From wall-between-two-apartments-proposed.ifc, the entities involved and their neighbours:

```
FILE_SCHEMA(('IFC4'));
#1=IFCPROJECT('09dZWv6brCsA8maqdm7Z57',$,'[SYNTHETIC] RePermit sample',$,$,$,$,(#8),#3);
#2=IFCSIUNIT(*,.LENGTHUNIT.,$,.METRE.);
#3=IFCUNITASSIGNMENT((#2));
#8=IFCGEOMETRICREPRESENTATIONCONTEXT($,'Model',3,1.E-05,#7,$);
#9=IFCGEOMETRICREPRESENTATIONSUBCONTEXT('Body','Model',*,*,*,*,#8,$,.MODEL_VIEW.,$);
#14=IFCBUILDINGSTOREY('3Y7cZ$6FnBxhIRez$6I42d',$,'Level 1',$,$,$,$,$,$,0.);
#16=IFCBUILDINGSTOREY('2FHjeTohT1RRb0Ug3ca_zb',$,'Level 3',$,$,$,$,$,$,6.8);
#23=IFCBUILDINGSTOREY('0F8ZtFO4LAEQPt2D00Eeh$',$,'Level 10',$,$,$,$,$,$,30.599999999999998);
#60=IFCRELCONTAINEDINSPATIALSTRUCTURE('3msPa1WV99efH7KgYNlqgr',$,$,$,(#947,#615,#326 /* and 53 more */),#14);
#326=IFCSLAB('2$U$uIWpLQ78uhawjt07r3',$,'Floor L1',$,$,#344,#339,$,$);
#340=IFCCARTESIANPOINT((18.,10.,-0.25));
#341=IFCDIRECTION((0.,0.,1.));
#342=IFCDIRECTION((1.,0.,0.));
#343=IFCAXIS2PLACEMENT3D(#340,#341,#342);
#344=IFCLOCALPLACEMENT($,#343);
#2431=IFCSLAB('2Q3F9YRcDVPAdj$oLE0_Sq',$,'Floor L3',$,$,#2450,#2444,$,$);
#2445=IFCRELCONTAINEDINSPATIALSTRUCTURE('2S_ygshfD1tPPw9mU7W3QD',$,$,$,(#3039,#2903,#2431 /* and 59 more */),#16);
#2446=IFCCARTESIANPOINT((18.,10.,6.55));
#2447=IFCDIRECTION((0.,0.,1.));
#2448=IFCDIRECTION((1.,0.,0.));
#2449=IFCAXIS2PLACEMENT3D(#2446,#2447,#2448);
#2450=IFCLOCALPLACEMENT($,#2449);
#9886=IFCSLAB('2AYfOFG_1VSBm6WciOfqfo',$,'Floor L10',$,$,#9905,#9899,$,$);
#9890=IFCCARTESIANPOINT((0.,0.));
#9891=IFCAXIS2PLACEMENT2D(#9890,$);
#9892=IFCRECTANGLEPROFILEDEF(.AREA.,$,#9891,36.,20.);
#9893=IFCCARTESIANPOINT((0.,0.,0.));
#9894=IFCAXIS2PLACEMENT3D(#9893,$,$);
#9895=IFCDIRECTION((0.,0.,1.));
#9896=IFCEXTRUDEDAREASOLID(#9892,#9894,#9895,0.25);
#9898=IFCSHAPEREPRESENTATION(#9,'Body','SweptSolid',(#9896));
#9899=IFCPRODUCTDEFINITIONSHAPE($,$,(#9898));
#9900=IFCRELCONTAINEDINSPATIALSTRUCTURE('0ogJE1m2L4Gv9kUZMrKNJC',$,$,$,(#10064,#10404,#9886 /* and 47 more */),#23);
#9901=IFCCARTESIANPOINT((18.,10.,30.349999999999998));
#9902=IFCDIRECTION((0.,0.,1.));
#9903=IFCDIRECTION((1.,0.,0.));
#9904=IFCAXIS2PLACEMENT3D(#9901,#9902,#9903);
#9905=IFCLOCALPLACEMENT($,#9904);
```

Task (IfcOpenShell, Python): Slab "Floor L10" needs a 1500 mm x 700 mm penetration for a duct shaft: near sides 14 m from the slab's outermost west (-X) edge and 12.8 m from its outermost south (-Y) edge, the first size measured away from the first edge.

```python
import numpy as np
import ifcopenshell
import ifcopenshell.api.feature
import ifcopenshell.api.geometry
import ifcopenshell.api.root
import ifcopenshell.geom
import ifcopenshell.util.placement
import ifcopenshell.util.representation
import ifcopenshell.util.shape
import ifcopenshell.util.unit

model = ifcopenshell.open("wall-between-two-apartments-proposed.ifc")
unit_scale = ifcopenshell.util.unit.calculate_unit_scale(model)
settings = ifcopenshell.geom.settings()


def volume(element):
    """Net volume in cubic metres, openings subtracted."""
    shape = ifcopenshell.geom.create_shape(settings, element)
    return ifcopenshell.util.shape.get_volume(shape.geometry)


slab = model.by_guid("2AYfOFG_1VSBm6WciOfqfo")
before = volume(slab)

# Extent in the slab's own axes, in metres. The edges named are its -X and -Y sides.
slab_shape = ifcopenshell.geom.create_shape(settings, slab)
vertices = ifcopenshell.util.shape.get_vertices(slab_shape.geometry)
x_min, y_min, bottom = vertices.min(axis=0)
top = vertices[:, 2].max()

opening = ifcopenshell.api.root.create_entity(model, ifc_class="IfcOpeningElement", name="Duct shaft opening", predefined_type="OPENING")
context = ifcopenshell.util.representation.get_context(model, "Model", "Body", "MODEL_VIEW")
width, depth = 1.5, 0.7
outline = [(0.0, 0.0), (width, 0.0), (width, depth), (0.0, depth), (0.0, 0.0)]
# Overshoot both faces by 50 mm so the cut is clean.
shape = ifcopenshell.api.geometry.add_slab_representation(
    model, context=context, depth=top - bottom + 0.1, polyline=outline
)
ifcopenshell.api.geometry.assign_representation(model, product=opening, representation=shape)

matrix = ifcopenshell.util.placement.get_local_placement(slab.ObjectPlacement)
matrix[:, 3] = matrix @ np.append(np.array([x_min + 14, y_min + 12.8, bottom - 0.05]) / unit_scale, 1.0)
ifcopenshell.api.geometry.edit_object_placement(model, product=opening, matrix=matrix, is_si=False)
ifcopenshell.api.feature.add_feature(model, feature=opening, element=slab)

after = volume(slab)

print(f"slab volume {before:.3f} -> {after:.3f} m3")

model.write("wall-between-two-apartments-proposed_v2.ifc")
```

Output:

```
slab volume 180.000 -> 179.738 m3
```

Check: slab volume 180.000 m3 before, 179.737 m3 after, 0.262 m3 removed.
